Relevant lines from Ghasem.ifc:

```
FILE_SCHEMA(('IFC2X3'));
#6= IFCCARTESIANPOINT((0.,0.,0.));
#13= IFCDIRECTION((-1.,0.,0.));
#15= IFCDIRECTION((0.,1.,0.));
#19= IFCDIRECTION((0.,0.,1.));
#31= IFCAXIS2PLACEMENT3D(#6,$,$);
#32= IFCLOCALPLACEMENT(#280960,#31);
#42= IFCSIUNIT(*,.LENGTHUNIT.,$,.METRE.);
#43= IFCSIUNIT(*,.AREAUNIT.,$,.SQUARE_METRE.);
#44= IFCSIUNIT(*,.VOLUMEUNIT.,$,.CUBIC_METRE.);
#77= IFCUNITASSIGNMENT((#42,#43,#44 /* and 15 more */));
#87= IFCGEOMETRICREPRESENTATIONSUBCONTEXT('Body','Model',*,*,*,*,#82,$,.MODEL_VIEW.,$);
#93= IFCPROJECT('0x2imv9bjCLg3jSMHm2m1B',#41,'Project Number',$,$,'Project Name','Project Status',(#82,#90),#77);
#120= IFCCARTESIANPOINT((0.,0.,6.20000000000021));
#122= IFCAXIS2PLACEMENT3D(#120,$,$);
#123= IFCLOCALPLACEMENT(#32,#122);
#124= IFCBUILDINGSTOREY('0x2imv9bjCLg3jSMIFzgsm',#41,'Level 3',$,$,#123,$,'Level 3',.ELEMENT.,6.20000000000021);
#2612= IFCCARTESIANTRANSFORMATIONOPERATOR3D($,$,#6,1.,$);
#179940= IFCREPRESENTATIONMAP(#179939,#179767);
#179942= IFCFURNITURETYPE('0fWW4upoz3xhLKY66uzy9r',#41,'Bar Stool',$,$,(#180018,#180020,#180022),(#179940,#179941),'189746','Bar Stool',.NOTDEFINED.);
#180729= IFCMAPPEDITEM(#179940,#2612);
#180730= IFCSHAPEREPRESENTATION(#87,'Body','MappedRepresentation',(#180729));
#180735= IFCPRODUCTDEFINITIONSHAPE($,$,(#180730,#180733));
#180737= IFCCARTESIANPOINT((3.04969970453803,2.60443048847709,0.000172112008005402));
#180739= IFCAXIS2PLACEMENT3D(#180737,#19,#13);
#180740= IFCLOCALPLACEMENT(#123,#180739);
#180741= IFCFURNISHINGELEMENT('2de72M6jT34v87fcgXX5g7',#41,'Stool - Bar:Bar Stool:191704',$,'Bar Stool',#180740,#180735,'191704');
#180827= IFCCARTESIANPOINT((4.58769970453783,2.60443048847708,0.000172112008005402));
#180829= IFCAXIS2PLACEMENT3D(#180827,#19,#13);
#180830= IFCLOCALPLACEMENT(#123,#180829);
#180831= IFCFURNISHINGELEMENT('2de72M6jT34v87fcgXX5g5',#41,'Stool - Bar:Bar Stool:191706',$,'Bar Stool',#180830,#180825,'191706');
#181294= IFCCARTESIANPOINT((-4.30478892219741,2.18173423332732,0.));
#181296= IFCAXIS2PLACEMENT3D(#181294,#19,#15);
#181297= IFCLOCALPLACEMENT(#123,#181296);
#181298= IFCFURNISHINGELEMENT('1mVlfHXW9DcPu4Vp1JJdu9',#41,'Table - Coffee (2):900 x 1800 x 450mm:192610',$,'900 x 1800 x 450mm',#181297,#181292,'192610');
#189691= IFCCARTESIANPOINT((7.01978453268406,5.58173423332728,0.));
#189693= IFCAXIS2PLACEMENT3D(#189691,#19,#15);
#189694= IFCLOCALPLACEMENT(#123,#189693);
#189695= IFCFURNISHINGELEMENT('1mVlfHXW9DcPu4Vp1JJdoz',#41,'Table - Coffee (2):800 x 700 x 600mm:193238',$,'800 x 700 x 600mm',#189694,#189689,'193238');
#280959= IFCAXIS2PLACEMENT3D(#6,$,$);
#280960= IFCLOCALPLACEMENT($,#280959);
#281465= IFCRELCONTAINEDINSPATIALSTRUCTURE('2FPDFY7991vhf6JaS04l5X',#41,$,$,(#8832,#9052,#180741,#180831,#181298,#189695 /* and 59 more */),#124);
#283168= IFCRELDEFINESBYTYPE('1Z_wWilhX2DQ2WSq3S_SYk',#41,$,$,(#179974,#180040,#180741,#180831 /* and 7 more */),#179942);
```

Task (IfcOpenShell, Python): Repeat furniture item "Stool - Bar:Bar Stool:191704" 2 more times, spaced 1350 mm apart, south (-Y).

```python
import numpy as np
import ifcopenshell
import ifcopenshell.api.geometry
import ifcopenshell.api.root
import ifcopenshell.util.element
import ifcopenshell.util.placement

model = ifcopenshell.open("Ghasem.ifc")


def reuse_history(source, copy):
    """copy_class also copies each property set's owner history, people and application; keep the originals."""
    for rel in copy.IsDefinedBy:
        if rel.is_a("IfcRelDefinesByProperties") and (history := rel.RelatingPropertyDefinition.OwnerHistory):
            rel.RelatingPropertyDefinition.OwnerHistory = source.OwnerHistory
            ifcopenshell.util.element.remove_deep2(model, history)


source = model.by_guid("2de72M6jT34v87fcgXX5g7")
base = ifcopenshell.util.placement.get_local_placement(source.ObjectPlacement)
step = np.array([0.0, -1.0, 0.0]) * 1.35

for i in range(1, 3):
    copy = ifcopenshell.api.root.copy_class(model, product=source)
    copy.Representation = ifcopenshell.util.element.copy_deep(
        model, source.Representation, exclude=["IfcGeometricRepresentationContext", "IfcRepresentationMap"]
    )
    copy.Name = "Stool - Bar:Bar Stool"
    copy.Tag = None
    reuse_history(source, copy)
    matrix = base.copy()
    matrix[:3, 3] += i * step
    print("added at", matrix[:3, 3].round(3) + 0.0)
    ifcopenshell.api.geometry.edit_object_placement(model, product=copy, matrix=matrix, is_si=False)

model.write("Ghasem-out.ifc")
```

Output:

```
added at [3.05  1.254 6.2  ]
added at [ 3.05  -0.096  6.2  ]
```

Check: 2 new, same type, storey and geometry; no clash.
